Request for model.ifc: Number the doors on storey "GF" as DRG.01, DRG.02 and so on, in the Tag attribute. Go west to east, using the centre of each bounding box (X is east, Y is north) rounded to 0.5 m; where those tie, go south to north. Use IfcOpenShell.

First a look at what the model holds.

```python
import ifcopenshell
import ifcopenshell.util.element
import ifcopenshell.util.placement

model = ifcopenshell.open("model.ifc")
print(model.schema)
storey = next(s for s in model.by_type("IfcBuildingStorey") if s.Name == "GF")
doors = [e for e in ifcopenshell.util.element.get_decomposition(storey) if e.is_a("IfcDoor")]
for e in sorted(doors, key=lambda e: e.id()):
    origin = ifcopenshell.util.placement.get_local_placement(e.ObjectPlacement)[:3, 3]
    print(e.id(), e.Tag, e.Name, origin.round(2) + 0.0, sep=" | ")
```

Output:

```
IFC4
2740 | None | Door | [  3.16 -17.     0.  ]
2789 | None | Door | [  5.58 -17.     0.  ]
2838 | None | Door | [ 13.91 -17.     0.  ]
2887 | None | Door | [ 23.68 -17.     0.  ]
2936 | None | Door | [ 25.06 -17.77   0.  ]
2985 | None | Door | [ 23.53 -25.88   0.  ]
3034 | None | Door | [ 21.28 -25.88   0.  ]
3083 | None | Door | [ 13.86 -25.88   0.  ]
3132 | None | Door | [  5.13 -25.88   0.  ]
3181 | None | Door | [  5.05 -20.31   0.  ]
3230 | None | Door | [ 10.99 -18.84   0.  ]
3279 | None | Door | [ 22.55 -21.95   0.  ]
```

```python
import ifcopenshell
import ifcopenshell.geom
import ifcopenshell.util.element
import ifcopenshell.util.shape

model = ifcopenshell.open("model.ifc")
settings = ifcopenshell.geom.settings()
settings.set("use-world-coords", True)


def centre(element):
    shape = ifcopenshell.geom.create_shape(settings, element)
    return ifcopenshell.util.shape.get_bbox_centroid(shape.geometry)


storey = next(s for s in model.by_type("IfcBuildingStorey") if s.Name == "GF")
doors = [e for e in ifcopenshell.util.element.get_decomposition(storey) if e.is_a("IfcDoor")]

# Insertion points can sit at a corner or the storey origin, so sort by the geometry (in metres).
centres = {e: centre(e) for e in doors}
doors.sort(key=lambda e: (round(centres[e][0] / 0.5), centres[e][1]))

for i, e in enumerate(doors, start=1):
    number = f"DRG.{i:02d}"
    e.Tag = number
    print(e.id(), number)

model.write("model_updated.ifc")
```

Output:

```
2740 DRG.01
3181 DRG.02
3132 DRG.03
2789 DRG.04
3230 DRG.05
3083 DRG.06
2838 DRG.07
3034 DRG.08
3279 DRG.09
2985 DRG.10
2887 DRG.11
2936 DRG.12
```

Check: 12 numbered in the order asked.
